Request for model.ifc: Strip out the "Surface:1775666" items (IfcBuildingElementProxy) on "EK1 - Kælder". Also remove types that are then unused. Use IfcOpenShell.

First a look at what the model holds.

```python
import ifcopenshell
import ifcopenshell.util.element

model = ifcopenshell.open("model.ifc")
print(model.schema)
storey = next(s for s in model.by_type("IfcBuildingStorey") if s.Name == "EK1 - Kælder")
proxies = [e for e in ifcopenshell.util.element.get_decomposition(storey) if e.is_a("IfcBuildingElementProxy")]
seen = {}
for e in proxies:
    element_type = ifcopenshell.util.element.get_type(e)
    name = element_type.Name if element_type not in (None, e) else None
    seen[name] = seen.get(name, 0) + 1
for name, count in sorted(seen.items(), key=str):
    print(count, "x", name)
```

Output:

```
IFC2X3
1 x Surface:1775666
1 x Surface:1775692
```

```python
import ifcopenshell
import ifcopenshell.api.root
import ifcopenshell.util.element

model = ifcopenshell.open("model.ifc")

storey = next(s for s in model.by_type("IfcBuildingStorey") if s.Name == "EK1 - Kælder")
proxies = [e for e in ifcopenshell.util.element.get_decomposition(storey) if e.is_a("IfcBuildingElementProxy")]
targets = [e for e in proxies if (t := ifcopenshell.util.element.get_type(e)) not in (None, e) and t.Name == "Surface:1775666"]
types = {ifcopenshell.util.element.get_type(e) for e in targets} - {None, *targets}

for e in targets:
    ifcopenshell.api.root.remove_product(model, product=e)
print(len(targets), "removed")

unused = [t for t in types if not ifcopenshell.util.element.get_types(t)]
for t in unused:
    ifcopenshell.api.root.remove_product(model, product=t)
print(len(unused), "unused types removed")

model.write("model_updated.ifc")
```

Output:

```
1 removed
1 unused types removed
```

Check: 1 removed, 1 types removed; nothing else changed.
